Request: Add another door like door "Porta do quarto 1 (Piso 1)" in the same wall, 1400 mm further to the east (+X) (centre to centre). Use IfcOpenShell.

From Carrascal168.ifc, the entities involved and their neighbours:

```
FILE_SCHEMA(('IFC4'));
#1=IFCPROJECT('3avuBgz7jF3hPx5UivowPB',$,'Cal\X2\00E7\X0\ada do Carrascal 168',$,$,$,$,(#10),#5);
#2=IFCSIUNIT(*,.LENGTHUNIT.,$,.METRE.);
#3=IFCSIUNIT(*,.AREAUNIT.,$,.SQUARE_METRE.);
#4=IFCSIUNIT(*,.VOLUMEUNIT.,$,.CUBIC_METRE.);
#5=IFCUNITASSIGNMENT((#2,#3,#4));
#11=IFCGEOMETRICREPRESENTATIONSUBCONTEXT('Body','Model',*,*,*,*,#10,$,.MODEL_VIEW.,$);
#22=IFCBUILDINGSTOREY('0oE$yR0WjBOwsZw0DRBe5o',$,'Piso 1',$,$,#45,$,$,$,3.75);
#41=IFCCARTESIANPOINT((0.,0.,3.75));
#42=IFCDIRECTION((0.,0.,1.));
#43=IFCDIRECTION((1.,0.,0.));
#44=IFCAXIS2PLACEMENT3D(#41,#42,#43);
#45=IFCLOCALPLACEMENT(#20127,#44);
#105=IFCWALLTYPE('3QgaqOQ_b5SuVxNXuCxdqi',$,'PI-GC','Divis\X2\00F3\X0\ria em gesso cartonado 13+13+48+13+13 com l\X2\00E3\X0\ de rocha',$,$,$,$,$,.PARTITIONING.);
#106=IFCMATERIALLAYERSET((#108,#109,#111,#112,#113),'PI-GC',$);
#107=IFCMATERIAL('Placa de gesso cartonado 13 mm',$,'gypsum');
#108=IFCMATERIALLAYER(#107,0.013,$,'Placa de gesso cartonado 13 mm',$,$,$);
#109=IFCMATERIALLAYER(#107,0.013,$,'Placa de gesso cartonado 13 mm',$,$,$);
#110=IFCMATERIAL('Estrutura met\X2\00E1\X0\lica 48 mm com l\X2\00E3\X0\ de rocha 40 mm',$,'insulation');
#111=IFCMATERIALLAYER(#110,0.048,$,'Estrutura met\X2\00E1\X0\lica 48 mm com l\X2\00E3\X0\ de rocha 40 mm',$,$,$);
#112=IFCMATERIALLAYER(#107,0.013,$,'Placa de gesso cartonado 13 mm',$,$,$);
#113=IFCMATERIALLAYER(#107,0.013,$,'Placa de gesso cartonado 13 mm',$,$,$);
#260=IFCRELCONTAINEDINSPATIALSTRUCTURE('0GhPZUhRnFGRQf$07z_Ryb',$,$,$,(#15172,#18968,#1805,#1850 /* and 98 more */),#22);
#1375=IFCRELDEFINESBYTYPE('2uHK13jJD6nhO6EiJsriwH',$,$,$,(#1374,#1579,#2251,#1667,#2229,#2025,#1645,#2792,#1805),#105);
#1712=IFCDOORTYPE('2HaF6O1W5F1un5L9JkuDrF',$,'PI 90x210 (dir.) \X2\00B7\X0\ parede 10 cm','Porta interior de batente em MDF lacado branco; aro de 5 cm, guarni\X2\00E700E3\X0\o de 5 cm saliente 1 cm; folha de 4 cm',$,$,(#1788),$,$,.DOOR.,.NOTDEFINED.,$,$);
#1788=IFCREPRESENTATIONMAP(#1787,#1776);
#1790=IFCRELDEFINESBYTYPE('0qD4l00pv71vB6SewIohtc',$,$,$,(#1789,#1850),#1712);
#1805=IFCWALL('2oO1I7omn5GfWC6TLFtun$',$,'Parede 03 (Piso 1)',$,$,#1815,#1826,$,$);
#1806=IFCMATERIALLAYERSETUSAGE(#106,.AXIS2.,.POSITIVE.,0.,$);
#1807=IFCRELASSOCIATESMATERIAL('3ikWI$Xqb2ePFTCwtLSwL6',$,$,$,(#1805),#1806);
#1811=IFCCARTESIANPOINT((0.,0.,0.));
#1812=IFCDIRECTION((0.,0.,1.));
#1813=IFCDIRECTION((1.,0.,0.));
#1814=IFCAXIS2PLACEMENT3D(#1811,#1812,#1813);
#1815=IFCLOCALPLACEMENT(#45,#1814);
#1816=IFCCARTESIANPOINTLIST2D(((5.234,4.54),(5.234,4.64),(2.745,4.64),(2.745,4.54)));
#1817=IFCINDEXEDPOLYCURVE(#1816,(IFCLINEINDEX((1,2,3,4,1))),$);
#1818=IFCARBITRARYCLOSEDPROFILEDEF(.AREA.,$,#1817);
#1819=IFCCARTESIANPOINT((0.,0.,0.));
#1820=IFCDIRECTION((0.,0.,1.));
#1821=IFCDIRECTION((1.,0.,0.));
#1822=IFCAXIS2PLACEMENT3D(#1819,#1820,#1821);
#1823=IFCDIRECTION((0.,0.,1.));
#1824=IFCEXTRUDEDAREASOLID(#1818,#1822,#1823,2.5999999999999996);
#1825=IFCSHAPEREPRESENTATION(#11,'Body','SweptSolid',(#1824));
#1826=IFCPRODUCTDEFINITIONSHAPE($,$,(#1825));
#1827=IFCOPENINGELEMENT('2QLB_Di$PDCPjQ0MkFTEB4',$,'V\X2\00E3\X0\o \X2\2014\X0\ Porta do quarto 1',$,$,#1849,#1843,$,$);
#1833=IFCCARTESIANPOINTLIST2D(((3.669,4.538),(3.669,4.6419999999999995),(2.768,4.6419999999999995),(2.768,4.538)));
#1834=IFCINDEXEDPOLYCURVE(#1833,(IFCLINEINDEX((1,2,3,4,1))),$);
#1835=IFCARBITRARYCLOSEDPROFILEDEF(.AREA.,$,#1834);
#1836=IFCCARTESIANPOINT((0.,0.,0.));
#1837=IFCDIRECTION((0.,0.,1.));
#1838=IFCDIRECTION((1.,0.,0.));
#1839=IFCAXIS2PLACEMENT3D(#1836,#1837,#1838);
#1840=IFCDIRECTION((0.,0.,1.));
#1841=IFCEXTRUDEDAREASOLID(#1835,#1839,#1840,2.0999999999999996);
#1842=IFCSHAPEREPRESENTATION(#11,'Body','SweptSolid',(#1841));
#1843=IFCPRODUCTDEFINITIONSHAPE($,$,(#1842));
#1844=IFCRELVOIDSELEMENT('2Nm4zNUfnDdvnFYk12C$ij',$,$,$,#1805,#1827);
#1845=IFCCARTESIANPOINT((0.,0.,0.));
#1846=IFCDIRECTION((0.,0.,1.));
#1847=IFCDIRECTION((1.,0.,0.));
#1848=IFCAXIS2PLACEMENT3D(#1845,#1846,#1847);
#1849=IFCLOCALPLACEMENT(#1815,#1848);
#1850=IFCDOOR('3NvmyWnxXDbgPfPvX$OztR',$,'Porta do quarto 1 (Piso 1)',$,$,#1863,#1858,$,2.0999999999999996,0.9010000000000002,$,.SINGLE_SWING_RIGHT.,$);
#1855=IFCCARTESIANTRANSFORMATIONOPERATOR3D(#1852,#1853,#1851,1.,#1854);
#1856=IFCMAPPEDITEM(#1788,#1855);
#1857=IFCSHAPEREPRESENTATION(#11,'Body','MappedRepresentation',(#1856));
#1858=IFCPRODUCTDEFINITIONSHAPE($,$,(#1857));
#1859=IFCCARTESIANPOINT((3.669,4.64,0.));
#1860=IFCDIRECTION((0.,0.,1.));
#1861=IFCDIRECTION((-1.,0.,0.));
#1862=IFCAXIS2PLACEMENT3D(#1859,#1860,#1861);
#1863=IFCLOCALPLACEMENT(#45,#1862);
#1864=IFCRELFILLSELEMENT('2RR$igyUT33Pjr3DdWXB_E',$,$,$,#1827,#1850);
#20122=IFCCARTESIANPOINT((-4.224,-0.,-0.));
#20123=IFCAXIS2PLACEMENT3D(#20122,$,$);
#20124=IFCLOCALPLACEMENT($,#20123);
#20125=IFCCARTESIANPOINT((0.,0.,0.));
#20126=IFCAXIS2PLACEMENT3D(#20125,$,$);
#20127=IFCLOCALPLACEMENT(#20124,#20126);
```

```python
import ifcopenshell
import ifcopenshell.api.feature
import ifcopenshell.api.geometry
import ifcopenshell.api.root
import ifcopenshell.geom
import ifcopenshell.util.element
import ifcopenshell.util.placement
import ifcopenshell.util.shape

model = ifcopenshell.open("Carrascal168.ifc")
settings = ifcopenshell.geom.settings()


def volume(element):
    """Net volume in cubic metres, openings subtracted."""
    shape = ifcopenshell.geom.create_shape(settings, element)
    return ifcopenshell.util.shape.get_volume(shape.geometry)


door = model.by_guid("3NvmyWnxXDbgPfPvX$OztR")
opening = door.FillsVoids[0].RelatingOpeningElement
wall = opening.VoidsElements[0].RelatingBuildingElement
before = volume(wall)
shift = ifcopenshell.util.placement.get_local_placement(wall.ObjectPlacement)[:3, 0] * 1.4

# copy_class copies the void relationship, type, container and properties, but no geometry.
new_opening = ifcopenshell.api.root.copy_class(model, product=opening)
new_opening.Representation = ifcopenshell.util.element.copy_deep(
    model, opening.Representation, exclude=["IfcGeometricRepresentationContext", "IfcRepresentationMap"]
)
new_door = ifcopenshell.api.root.copy_class(model, product=door)
new_door.Representation = ifcopenshell.util.element.copy_deep(
    model, door.Representation, exclude=["IfcGeometricRepresentationContext", "IfcRepresentationMap"]
)
ifcopenshell.api.feature.add_filling(model, opening=new_opening, element=new_door)

for old, new in ((opening, new_opening), (door, new_door)):
    matrix = ifcopenshell.util.placement.get_local_placement(old.ObjectPlacement)
    matrix[:3, 3] += shift
    ifcopenshell.api.geometry.edit_object_placement(model, product=new, matrix=matrix, is_si=False)

after = volume(wall)

print(f"wall volume {before:.3f} -> {after:.3f} m3")

model.write("Carrascal168_rev.ifc")
```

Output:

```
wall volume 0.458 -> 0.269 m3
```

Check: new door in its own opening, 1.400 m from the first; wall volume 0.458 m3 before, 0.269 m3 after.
